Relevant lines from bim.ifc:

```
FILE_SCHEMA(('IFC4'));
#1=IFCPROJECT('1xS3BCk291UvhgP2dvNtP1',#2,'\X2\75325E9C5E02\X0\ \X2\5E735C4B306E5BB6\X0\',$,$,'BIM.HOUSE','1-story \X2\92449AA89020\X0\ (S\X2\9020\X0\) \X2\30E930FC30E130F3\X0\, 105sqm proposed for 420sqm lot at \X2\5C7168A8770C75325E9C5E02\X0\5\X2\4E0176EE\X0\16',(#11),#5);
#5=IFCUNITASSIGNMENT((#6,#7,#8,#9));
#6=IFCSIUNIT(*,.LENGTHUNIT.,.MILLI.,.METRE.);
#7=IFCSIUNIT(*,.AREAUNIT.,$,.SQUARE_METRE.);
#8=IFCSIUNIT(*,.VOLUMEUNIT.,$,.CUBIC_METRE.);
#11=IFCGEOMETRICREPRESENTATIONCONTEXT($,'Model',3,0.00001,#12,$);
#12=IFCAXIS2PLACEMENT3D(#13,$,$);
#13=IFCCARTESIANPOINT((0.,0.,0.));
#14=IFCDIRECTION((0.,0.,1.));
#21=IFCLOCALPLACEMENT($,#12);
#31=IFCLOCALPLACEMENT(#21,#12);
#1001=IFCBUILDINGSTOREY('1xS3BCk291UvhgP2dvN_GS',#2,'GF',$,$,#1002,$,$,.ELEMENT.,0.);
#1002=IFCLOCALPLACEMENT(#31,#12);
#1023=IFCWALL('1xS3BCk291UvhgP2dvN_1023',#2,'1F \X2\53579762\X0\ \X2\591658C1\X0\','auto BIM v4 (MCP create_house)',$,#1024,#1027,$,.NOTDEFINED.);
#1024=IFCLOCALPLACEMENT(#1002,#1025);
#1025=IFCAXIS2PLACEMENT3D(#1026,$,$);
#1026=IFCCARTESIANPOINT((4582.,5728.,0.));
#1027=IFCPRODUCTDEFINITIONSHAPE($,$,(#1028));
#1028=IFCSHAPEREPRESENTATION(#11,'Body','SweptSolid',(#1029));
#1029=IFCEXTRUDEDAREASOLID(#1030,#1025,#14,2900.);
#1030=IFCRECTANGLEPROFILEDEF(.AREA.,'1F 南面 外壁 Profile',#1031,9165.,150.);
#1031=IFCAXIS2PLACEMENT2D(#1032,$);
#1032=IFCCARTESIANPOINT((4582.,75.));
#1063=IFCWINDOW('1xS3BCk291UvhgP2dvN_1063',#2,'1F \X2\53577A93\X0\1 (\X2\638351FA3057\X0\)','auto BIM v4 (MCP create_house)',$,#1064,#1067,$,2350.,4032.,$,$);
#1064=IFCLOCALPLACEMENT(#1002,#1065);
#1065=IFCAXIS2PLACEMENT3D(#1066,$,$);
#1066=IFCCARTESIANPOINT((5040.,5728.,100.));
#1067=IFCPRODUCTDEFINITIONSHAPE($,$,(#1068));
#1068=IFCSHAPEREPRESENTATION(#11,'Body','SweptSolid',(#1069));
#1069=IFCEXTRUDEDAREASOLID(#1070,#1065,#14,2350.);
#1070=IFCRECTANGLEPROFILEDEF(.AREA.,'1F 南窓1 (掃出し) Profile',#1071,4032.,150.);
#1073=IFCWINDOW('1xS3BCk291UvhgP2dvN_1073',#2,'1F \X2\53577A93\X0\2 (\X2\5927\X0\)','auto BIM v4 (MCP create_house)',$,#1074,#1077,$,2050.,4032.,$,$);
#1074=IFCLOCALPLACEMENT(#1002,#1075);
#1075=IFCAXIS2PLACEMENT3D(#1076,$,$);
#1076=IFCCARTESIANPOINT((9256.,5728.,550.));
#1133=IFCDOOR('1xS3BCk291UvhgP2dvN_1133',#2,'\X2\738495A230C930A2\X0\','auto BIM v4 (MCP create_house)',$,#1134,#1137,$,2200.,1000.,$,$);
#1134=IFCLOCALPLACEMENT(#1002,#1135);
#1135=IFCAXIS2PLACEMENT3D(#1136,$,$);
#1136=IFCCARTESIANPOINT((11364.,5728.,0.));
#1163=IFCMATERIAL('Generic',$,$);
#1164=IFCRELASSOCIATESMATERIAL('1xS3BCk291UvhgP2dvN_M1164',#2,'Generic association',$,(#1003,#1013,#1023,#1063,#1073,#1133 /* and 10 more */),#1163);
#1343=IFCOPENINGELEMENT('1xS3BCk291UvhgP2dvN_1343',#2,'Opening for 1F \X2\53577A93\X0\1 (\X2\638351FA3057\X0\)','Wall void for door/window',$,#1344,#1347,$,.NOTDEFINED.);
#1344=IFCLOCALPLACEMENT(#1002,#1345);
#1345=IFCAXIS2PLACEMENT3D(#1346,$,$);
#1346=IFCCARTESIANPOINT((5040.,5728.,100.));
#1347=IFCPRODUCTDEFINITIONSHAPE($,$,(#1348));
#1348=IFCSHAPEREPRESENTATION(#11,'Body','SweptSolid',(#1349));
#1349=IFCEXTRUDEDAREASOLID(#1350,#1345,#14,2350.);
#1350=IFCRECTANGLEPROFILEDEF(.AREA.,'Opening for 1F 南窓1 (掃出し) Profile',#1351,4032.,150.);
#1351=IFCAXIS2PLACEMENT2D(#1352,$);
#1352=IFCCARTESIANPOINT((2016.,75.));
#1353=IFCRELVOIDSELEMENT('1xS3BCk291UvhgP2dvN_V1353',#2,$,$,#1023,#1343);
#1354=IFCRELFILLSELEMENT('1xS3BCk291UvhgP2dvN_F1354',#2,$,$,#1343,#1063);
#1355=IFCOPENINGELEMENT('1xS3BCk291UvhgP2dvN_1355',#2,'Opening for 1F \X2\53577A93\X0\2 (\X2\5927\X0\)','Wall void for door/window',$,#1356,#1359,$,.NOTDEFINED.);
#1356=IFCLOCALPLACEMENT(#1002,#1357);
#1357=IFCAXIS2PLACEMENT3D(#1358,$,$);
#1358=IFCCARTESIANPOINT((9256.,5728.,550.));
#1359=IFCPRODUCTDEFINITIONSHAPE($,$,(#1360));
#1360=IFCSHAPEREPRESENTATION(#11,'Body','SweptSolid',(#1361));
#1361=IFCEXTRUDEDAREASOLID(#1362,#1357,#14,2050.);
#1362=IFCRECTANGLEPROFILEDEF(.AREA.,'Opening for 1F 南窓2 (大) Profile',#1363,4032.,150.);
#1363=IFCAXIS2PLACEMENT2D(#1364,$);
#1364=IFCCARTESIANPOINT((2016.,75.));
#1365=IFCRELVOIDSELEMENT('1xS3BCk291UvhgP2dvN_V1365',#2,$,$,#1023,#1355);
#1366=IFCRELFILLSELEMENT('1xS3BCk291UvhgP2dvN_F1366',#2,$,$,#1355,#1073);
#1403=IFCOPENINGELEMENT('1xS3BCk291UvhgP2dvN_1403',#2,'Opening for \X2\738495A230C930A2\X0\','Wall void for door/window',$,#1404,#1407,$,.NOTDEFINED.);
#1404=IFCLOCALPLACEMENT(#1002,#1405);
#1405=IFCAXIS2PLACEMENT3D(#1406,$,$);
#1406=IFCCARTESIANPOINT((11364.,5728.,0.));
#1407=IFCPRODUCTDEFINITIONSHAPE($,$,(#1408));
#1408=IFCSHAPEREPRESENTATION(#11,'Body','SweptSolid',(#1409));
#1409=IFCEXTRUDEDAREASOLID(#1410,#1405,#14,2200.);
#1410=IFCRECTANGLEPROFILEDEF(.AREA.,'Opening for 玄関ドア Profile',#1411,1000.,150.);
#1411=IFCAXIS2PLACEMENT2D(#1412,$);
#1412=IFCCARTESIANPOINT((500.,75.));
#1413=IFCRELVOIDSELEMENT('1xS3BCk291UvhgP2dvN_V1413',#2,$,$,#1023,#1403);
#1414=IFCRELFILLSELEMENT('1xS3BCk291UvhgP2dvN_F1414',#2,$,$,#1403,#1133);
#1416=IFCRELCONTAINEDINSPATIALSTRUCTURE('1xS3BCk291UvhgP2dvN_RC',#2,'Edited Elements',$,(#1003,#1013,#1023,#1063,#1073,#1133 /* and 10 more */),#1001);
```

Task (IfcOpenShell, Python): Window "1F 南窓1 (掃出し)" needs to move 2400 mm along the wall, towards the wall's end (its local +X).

```python
import ifcopenshell
import ifcopenshell.api.geometry
import ifcopenshell.util.placement

model = ifcopenshell.open("bim.ifc")

window = model.by_guid("1xS3BCk291UvhgP2dvN_1063")
opening = window.FillsVoids[0].RelatingOpeningElement
wall = opening.VoidsElements[0].RelatingBuildingElement

wall_matrix = ifcopenshell.util.placement.get_local_placement(wall.ObjectPlacement)
shift = wall_matrix[:3, 0] * 2400.0
before = ifcopenshell.util.placement.get_local_placement(window.ObjectPlacement)[:3, 3].copy()

# The window is not placed relative to its opening, so move both.
for product in (opening, window):
    matrix = ifcopenshell.util.placement.get_local_placement(product.ObjectPlacement)
    matrix[:3, 3] += shift
    ifcopenshell.api.geometry.edit_object_placement(model, product=product, matrix=matrix, is_si=False)

after = ifcopenshell.util.placement.get_local_placement(window.ObjectPlacement)[:3, 3]
print("window moved by", (after - before).round(3) + 0.0)

model.write("bim_v2.ifc")
```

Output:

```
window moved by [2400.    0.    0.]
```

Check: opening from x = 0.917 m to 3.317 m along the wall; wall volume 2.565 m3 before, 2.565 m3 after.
